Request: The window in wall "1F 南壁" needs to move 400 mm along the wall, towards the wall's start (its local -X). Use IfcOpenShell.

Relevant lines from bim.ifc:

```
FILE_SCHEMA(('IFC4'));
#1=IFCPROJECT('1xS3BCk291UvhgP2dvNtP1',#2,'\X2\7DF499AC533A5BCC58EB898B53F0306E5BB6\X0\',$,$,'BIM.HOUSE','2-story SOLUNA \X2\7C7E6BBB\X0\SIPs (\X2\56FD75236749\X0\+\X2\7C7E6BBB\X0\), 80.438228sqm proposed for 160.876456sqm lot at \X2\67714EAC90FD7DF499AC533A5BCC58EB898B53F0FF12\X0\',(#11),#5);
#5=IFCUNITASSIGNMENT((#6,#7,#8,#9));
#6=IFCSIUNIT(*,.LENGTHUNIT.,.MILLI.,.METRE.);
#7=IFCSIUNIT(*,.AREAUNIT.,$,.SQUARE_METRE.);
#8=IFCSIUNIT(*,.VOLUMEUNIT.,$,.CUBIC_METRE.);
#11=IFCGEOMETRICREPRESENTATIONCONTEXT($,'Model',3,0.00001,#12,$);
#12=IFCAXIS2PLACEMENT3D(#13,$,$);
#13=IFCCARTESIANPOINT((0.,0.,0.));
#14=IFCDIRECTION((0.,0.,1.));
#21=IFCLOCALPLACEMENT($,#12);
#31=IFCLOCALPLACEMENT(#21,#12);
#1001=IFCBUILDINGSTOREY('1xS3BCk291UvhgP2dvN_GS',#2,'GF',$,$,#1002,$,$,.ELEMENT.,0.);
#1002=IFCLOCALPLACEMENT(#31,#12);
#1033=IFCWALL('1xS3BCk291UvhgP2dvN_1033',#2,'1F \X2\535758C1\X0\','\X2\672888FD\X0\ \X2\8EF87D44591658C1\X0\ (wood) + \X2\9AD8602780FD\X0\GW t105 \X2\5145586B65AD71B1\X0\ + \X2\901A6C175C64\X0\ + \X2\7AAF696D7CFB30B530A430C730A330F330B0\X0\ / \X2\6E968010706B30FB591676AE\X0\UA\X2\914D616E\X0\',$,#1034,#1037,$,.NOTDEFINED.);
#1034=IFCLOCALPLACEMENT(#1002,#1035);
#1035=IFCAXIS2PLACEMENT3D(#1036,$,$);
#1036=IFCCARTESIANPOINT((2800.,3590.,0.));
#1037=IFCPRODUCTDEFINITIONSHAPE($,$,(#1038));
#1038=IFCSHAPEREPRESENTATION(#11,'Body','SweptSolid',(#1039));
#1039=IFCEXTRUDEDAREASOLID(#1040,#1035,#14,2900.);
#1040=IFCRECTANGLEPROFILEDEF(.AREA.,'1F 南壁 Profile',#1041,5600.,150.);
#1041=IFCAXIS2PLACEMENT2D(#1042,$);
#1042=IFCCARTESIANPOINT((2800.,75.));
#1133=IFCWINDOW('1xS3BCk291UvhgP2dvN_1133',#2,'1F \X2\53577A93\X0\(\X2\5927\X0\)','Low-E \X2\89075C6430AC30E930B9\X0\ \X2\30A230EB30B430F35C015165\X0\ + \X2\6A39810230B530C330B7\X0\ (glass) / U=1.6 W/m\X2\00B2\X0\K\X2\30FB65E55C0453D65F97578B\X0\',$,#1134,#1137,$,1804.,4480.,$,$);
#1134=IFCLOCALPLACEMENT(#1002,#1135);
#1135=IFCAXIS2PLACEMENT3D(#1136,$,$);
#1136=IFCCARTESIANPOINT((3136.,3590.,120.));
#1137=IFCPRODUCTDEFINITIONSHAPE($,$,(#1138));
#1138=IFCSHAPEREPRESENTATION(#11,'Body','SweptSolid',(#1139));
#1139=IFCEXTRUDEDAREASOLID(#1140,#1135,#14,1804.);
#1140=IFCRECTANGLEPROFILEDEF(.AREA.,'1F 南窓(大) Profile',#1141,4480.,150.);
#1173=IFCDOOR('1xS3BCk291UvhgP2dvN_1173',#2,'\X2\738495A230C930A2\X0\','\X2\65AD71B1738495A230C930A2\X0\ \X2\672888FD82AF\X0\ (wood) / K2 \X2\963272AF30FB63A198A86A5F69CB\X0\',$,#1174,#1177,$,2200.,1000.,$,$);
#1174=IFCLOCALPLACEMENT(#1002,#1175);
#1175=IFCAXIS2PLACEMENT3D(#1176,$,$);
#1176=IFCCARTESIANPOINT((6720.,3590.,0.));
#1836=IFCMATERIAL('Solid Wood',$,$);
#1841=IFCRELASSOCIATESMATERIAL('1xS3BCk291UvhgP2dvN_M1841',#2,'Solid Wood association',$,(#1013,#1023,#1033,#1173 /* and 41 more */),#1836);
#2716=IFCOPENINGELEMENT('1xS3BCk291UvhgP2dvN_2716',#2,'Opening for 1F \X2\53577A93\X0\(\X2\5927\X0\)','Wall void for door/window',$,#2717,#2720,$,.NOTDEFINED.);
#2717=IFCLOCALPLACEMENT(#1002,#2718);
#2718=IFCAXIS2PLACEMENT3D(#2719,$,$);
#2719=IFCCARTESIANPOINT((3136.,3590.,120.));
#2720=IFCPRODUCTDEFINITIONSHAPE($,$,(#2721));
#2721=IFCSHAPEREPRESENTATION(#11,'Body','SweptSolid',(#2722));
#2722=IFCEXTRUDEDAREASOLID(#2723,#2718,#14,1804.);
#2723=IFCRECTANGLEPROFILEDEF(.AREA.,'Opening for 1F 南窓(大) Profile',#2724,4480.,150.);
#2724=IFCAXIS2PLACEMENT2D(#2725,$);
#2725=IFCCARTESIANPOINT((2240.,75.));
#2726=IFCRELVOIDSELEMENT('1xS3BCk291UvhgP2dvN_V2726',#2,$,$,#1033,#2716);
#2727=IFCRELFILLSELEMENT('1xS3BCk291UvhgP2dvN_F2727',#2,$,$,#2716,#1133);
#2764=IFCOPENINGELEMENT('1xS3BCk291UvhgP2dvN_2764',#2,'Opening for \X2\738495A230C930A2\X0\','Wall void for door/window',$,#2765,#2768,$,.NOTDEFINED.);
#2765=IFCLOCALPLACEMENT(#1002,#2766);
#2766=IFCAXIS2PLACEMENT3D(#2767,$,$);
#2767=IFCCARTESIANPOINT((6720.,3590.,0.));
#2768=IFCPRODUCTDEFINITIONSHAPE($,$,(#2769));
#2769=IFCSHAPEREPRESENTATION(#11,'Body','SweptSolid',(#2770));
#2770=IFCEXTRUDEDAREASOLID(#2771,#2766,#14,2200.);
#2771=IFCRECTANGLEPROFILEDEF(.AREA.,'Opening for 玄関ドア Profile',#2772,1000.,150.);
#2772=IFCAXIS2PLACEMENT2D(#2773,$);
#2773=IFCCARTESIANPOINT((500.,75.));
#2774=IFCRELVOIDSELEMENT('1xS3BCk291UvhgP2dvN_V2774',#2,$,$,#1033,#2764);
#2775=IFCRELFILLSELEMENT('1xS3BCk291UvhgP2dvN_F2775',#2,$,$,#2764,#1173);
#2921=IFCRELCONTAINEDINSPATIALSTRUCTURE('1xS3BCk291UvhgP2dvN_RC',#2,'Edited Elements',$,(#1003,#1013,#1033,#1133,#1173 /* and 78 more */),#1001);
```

```python
import ifcopenshell
import ifcopenshell.api.geometry
import ifcopenshell.util.placement
import ifcopenshell.util.unit

model = ifcopenshell.open("bim.ifc")
unit_scale = ifcopenshell.util.unit.calculate_unit_scale(model)

window = model.by_guid("1xS3BCk291UvhgP2dvN_1133")
opening = window.FillsVoids[0].RelatingOpeningElement
wall = opening.VoidsElements[0].RelatingBuildingElement

wall_matrix = ifcopenshell.util.placement.get_local_placement(wall.ObjectPlacement)
shift = wall_matrix[:3, 0] * -0.4 / unit_scale
before = ifcopenshell.util.placement.get_local_placement(window.ObjectPlacement)[:3, 3].copy()

# The window is not placed relative to its opening, so move both.
for product in (opening, window):
    matrix = ifcopenshell.util.placement.get_local_placement(product.ObjectPlacement)
    matrix[:3, 3] += shift
    ifcopenshell.api.geometry.edit_object_placement(model, product=product, matrix=matrix, is_si=False)

after = ifcopenshell.util.placement.get_local_placement(window.ObjectPlacement)[:3, 3]
print("window moved by", (after - before).round(3) + 0.0)

model.write("bim_updated.ifc")
```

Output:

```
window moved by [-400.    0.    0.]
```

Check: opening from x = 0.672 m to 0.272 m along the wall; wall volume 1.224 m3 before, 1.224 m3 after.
